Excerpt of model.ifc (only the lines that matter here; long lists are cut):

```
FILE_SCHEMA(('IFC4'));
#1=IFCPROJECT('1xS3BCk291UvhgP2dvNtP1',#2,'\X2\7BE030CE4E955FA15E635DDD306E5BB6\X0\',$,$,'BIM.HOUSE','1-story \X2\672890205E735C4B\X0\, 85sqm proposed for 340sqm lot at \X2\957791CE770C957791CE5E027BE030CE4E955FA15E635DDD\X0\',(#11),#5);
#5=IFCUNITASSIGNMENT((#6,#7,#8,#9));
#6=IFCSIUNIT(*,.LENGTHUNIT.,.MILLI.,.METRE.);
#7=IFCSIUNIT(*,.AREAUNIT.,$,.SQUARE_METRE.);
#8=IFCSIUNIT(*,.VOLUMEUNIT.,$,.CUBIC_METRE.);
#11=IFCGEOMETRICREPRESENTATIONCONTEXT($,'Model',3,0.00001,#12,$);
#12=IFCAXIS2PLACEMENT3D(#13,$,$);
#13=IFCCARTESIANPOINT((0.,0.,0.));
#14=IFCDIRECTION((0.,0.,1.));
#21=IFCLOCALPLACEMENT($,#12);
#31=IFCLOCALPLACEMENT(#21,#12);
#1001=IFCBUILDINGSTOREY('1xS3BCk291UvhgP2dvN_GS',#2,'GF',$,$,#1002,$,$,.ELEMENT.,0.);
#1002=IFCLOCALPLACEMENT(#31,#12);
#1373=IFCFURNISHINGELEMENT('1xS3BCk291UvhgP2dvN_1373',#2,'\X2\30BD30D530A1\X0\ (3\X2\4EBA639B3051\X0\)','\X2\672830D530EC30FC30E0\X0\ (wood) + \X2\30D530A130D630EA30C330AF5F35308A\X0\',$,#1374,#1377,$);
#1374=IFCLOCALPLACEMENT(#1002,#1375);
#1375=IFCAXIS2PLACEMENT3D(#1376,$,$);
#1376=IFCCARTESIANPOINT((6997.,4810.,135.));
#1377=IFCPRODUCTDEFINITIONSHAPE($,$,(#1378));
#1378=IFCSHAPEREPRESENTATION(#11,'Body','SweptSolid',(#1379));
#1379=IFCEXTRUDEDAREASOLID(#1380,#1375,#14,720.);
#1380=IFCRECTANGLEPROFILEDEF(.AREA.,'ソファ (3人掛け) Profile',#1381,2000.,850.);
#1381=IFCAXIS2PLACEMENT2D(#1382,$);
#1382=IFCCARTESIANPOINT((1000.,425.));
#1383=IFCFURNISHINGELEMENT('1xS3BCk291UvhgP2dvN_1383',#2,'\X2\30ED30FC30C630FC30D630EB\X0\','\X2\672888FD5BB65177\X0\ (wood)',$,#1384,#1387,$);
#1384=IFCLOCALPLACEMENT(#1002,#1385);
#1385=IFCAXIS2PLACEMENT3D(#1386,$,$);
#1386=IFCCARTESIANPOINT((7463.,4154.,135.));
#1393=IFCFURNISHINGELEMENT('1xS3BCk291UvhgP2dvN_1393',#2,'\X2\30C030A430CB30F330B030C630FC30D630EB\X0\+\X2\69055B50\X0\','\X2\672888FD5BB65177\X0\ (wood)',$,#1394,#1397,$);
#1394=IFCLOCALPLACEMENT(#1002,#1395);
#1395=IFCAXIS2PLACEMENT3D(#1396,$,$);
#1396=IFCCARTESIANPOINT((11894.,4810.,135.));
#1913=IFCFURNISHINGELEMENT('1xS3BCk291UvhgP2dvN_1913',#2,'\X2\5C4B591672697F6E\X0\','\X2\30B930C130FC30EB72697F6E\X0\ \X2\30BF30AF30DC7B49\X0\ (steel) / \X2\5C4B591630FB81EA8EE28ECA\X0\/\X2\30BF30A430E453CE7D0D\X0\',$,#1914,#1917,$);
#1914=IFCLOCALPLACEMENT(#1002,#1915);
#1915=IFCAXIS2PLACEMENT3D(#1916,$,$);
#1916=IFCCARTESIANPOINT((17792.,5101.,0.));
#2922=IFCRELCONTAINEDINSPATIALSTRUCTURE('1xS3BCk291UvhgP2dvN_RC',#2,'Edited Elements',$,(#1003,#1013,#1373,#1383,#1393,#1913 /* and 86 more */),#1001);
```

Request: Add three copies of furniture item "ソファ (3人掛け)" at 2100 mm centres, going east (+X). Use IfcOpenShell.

```python
import numpy as np
import ifcopenshell
import ifcopenshell.api.geometry
import ifcopenshell.api.root
import ifcopenshell.util.element
import ifcopenshell.util.placement
import ifcopenshell.util.unit

model = ifcopenshell.open("model.ifc")
unit_scale = ifcopenshell.util.unit.calculate_unit_scale(model)


def reuse_history(source, copy):
    """copy_class also copies each property set's owner history, people and application; keep the originals."""
    for rel in copy.IsDefinedBy:
        if rel.is_a("IfcRelDefinesByProperties") and (history := rel.RelatingPropertyDefinition.OwnerHistory):
            rel.RelatingPropertyDefinition.OwnerHistory = source.OwnerHistory
            ifcopenshell.util.element.remove_deep2(model, history)


source = model.by_guid("1xS3BCk291UvhgP2dvN_1373")
base = ifcopenshell.util.placement.get_local_placement(source.ObjectPlacement)
step = np.array([1.0, 0.0, 0.0]) * 2.1 / unit_scale

for i in range(1, 4):
    copy = ifcopenshell.api.root.copy_class(model, product=source)
    copy.Representation = ifcopenshell.util.element.copy_deep(
        model, source.Representation, exclude=["IfcGeometricRepresentationContext", "IfcRepresentationMap"]
    )
    reuse_history(source, copy)
    matrix = base.copy()
    matrix[:3, 3] += i * step
    print("added at", matrix[:3, 3].round(3) + 0.0)
    ifcopenshell.api.geometry.edit_object_placement(model, product=copy, matrix=matrix, is_si=False)

model.write("model_edited.ifc")
```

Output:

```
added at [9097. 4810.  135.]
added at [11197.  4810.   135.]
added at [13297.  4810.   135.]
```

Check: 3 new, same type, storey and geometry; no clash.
